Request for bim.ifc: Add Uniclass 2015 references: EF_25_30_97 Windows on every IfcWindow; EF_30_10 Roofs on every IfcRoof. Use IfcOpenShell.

First a look at what the model holds.

```python
import ifcopenshell

model = ifcopenshell.open("bim.ifc")
print(model.schema)
print("classifications:", [c.Name for c in model.by_type("IfcClassification")])
for ifc_class in ("IfcDoor", "IfcRoof", "IfcStair", "IfcWall", "IfcWindow"):
    print(ifc_class, len(model.by_type(ifc_class)))
```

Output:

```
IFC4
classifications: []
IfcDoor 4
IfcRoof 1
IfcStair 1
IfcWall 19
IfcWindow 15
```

```python
import ifcopenshell
import ifcopenshell.api.classification

model = ifcopenshell.open("bim.ifc")

system = ifcopenshell.api.classification.add_classification(model, classification="Uniclass 2015")

codes = {
    "IfcWindow": ("EF_25_30_97", "Windows"),
    "IfcRoof": ("EF_30_10", "Roofs"),
}
for ifc_class, (code, name) in codes.items():
    products = model.by_type(ifc_class)
    ifcopenshell.api.classification.add_reference(
        model, products=products, classification=system, identification=code, name=name
    )
    print(code, len(products))

model.write("bim_updated.ifc")
```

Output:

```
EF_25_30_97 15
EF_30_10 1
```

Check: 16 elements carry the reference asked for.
